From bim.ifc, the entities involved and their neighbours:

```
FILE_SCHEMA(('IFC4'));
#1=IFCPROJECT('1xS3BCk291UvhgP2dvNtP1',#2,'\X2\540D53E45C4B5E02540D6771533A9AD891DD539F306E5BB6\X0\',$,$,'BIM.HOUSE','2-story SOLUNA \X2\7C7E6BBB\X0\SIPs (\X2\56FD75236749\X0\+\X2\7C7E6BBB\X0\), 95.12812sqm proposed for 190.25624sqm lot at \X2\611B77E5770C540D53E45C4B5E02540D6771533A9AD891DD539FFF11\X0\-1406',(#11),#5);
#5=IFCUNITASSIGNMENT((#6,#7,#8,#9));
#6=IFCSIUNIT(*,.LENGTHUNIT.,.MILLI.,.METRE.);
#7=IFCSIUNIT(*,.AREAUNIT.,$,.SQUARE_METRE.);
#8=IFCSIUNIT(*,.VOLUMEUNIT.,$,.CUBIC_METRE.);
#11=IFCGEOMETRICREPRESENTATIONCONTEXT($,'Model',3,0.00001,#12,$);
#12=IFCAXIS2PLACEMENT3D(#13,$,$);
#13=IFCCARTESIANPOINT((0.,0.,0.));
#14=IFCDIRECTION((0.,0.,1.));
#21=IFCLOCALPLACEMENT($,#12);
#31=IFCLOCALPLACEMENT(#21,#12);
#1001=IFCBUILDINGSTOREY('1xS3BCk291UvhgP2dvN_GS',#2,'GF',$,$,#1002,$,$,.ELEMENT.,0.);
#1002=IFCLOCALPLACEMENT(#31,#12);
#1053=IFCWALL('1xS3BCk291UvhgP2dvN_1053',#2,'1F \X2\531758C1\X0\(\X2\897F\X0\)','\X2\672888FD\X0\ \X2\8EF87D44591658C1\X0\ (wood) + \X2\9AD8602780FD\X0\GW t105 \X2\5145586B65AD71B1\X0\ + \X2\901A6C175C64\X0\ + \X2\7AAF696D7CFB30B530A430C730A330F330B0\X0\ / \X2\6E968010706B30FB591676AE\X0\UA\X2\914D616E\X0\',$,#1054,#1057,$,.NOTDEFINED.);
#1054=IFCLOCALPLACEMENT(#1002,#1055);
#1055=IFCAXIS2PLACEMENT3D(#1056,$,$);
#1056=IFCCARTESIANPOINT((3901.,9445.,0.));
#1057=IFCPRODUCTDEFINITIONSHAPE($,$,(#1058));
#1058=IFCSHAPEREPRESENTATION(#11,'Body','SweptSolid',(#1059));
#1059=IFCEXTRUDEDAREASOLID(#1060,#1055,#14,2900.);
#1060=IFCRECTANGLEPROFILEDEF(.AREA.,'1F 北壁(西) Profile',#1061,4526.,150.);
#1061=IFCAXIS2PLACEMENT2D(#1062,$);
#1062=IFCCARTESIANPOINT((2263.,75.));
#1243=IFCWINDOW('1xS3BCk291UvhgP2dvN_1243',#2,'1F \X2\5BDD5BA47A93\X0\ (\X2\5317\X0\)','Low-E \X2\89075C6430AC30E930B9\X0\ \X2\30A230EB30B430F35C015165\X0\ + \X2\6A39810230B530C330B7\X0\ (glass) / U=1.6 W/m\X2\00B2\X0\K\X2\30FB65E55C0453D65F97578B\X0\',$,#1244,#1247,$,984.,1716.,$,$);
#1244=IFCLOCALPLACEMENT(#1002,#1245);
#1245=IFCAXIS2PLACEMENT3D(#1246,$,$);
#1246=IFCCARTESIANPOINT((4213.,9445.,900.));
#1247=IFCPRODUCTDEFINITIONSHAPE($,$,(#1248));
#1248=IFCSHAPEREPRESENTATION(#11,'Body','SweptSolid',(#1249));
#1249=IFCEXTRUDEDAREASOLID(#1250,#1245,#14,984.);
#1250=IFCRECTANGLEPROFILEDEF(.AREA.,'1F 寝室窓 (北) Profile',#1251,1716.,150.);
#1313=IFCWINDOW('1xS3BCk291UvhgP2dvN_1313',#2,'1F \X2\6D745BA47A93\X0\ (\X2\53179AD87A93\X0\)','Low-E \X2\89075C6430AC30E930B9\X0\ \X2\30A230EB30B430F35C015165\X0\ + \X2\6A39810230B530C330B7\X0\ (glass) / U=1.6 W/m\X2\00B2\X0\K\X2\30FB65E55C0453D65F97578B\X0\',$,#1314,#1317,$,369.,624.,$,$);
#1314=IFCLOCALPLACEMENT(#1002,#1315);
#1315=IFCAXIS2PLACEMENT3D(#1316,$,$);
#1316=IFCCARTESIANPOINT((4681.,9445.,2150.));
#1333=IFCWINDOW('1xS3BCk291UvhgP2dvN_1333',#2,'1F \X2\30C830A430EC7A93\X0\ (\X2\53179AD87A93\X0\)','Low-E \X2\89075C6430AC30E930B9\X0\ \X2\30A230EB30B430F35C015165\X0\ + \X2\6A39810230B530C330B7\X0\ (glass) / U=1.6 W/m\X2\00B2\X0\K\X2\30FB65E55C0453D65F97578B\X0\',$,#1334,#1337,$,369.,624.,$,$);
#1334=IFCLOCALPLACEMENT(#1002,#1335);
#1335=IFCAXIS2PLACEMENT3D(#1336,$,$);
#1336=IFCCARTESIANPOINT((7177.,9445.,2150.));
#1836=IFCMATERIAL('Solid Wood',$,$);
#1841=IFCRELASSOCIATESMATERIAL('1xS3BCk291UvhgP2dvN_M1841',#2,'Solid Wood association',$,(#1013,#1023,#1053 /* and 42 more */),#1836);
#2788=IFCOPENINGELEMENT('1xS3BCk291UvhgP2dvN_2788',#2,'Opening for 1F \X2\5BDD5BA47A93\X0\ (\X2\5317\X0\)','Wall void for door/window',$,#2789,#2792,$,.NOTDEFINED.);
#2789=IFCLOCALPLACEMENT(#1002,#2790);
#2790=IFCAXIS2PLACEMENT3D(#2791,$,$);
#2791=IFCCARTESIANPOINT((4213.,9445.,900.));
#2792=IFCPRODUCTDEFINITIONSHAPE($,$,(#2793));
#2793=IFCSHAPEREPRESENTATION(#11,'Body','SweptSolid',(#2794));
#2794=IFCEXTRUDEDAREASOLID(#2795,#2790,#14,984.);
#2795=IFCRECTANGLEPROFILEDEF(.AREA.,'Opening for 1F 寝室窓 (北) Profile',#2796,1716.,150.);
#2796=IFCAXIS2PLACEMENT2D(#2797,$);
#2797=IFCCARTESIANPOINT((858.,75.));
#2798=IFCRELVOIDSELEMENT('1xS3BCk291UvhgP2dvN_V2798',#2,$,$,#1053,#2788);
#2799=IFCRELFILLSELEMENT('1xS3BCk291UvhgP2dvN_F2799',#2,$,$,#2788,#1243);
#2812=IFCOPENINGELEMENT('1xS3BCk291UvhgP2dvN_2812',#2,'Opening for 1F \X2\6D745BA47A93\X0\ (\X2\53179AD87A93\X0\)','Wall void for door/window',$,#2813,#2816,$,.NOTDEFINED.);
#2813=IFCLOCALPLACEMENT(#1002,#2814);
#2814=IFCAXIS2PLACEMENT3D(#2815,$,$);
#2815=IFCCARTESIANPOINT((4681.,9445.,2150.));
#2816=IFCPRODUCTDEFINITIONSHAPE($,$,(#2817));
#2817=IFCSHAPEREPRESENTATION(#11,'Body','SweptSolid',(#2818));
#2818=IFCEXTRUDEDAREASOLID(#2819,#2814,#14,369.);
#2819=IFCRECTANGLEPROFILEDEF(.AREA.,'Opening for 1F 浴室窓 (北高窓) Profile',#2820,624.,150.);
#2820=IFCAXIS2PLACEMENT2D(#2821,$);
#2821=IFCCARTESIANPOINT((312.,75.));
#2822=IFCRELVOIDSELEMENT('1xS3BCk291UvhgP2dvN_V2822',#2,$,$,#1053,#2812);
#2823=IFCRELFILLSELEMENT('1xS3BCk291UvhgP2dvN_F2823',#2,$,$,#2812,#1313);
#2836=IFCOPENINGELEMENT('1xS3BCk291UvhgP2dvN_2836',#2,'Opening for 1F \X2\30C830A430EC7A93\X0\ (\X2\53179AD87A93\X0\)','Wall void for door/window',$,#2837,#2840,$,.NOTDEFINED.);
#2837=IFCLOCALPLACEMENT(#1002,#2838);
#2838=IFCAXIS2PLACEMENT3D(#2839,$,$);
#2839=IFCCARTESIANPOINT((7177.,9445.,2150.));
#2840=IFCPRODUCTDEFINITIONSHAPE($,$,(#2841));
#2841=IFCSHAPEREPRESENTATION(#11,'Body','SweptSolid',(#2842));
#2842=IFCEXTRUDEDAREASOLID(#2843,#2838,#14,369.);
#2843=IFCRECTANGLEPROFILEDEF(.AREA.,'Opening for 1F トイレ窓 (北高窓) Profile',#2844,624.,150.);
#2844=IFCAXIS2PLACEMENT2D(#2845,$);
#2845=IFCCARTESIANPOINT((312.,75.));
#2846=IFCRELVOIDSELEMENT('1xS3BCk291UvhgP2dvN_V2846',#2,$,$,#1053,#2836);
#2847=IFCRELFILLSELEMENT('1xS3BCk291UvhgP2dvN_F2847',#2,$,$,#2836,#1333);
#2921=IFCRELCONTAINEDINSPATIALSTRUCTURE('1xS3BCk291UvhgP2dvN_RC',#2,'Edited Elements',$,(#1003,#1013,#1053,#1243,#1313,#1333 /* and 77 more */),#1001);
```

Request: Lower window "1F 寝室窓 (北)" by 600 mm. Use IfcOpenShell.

```python
import numpy as np
import ifcopenshell
import ifcopenshell.api.geometry
import ifcopenshell.util.placement
import ifcopenshell.util.unit

model = ifcopenshell.open("bim.ifc")
unit_scale = ifcopenshell.util.unit.calculate_unit_scale(model)

window = model.by_guid("1xS3BCk291UvhgP2dvN_1243")
opening = window.FillsVoids[0].RelatingOpeningElement
dz = -0.6 / unit_scale

shift = np.array([0.0, 0.0, dz])
# The window is not placed relative to its opening, so move both.
for product in (opening, window):
    matrix = ifcopenshell.util.placement.get_local_placement(product.ObjectPlacement)
    matrix[:3, 3] += shift
    ifcopenshell.api.geometry.edit_object_placement(model, product=product, matrix=matrix, is_si=False)

print(f"moved by {dz * unit_scale:+.3f} m")

model.write("bim_edited.ifc")
```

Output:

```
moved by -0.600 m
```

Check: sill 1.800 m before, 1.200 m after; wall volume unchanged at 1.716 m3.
